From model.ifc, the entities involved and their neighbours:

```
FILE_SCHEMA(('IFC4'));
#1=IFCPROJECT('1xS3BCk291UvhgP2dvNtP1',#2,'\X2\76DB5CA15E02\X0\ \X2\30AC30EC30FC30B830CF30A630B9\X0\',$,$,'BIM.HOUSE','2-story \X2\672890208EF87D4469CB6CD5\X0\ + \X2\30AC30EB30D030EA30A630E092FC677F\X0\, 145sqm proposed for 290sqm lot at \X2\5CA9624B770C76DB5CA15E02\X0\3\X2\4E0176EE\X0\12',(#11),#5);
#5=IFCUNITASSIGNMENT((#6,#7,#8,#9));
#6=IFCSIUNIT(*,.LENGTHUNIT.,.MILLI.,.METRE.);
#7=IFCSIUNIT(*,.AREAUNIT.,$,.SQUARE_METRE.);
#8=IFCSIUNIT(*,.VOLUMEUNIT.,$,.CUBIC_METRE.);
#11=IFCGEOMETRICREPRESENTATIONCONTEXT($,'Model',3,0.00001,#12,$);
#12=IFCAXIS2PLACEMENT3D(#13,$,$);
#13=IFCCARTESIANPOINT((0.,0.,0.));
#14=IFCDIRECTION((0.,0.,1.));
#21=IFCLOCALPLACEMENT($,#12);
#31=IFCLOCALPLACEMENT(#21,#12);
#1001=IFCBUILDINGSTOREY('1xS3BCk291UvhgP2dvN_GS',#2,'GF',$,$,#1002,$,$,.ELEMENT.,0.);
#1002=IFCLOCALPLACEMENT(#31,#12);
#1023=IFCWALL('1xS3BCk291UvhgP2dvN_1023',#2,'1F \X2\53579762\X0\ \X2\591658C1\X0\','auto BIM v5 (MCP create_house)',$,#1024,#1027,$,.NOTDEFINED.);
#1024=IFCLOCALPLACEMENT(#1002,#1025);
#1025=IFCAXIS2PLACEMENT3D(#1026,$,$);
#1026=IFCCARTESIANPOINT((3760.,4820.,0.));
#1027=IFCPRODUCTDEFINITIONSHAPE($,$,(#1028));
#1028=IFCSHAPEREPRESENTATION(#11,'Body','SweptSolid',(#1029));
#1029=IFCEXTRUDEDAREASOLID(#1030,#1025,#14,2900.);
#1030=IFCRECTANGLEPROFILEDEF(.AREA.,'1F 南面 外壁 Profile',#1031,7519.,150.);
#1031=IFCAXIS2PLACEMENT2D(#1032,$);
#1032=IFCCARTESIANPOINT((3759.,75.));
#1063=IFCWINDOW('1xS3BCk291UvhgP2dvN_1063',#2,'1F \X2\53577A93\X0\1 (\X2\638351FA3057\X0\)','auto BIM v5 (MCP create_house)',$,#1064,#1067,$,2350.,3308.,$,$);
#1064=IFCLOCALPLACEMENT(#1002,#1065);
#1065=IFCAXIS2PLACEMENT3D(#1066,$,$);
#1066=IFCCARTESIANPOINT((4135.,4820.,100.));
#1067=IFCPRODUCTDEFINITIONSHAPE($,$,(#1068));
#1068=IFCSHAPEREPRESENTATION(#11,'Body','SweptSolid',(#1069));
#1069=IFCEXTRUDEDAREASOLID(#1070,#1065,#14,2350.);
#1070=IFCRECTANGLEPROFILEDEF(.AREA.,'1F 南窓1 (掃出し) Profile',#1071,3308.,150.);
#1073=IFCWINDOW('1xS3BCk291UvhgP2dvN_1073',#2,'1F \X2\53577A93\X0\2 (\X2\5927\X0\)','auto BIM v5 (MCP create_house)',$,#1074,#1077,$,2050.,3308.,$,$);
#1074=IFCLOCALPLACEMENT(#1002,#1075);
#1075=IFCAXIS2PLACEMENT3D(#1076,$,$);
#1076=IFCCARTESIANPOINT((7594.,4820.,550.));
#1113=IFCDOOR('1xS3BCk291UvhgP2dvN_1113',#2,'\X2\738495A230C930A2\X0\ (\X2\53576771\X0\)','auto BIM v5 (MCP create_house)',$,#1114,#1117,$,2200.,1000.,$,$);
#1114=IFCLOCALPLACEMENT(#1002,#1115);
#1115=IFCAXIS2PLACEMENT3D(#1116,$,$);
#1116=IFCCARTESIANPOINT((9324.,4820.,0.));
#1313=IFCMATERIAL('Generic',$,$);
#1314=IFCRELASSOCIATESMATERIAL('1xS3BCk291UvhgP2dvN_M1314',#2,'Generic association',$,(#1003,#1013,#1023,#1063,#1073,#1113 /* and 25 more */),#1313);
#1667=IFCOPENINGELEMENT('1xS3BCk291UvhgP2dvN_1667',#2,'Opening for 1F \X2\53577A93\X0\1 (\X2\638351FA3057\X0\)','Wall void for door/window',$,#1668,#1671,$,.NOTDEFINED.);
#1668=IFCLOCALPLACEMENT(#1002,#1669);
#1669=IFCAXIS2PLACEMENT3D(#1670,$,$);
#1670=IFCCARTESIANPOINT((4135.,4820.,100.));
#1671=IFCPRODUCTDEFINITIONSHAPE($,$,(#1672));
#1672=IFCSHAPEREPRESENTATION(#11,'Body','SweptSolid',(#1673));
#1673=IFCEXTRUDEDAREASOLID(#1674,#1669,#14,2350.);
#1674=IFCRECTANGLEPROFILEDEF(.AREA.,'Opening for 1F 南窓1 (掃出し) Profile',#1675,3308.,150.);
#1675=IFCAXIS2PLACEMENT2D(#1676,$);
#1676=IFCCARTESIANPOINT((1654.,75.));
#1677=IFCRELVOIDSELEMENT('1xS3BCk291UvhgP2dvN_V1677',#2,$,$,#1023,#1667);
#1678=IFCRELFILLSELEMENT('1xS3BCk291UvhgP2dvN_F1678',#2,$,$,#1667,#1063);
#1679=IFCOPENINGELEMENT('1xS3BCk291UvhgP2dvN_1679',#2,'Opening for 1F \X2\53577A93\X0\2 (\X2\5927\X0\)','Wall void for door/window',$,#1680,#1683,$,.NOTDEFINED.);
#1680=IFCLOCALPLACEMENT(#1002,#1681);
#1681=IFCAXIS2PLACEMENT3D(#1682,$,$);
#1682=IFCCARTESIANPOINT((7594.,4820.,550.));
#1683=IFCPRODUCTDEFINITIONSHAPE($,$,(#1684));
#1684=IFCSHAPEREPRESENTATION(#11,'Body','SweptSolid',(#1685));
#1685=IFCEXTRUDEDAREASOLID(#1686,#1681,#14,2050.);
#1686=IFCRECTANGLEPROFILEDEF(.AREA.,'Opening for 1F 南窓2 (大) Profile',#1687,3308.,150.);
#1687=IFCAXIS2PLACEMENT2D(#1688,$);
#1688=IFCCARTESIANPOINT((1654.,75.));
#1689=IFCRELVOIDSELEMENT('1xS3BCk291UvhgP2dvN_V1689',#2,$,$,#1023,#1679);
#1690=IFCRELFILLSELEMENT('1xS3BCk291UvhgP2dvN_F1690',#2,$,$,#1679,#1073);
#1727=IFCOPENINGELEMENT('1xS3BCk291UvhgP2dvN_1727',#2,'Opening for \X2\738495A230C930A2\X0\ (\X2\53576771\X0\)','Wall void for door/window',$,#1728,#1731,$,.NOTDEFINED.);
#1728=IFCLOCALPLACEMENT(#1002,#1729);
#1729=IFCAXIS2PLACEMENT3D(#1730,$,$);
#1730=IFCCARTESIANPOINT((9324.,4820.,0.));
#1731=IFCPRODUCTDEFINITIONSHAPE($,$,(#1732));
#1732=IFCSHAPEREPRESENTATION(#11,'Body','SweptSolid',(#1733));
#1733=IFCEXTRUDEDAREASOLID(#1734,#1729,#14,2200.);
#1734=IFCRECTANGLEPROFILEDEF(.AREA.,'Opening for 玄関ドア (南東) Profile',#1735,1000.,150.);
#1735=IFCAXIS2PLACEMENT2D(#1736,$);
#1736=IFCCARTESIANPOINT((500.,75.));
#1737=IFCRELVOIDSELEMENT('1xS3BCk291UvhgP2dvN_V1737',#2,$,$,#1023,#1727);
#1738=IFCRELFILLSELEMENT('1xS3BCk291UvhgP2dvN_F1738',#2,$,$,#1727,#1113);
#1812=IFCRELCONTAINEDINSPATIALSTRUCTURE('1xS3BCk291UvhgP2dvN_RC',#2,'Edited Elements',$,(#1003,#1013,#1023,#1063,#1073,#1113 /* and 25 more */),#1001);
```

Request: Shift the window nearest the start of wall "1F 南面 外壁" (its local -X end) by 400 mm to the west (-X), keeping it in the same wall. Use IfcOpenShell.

```python
import ifcopenshell
import ifcopenshell.api.geometry
import ifcopenshell.util.placement

model = ifcopenshell.open("model.ifc")

window = model.by_id(1063)
opening = window.FillsVoids[0].RelatingOpeningElement
wall = opening.VoidsElements[0].RelatingBuildingElement

wall_matrix = ifcopenshell.util.placement.get_local_placement(wall.ObjectPlacement)
shift = wall_matrix[:3, 0] * -400.0
before = ifcopenshell.util.placement.get_local_placement(window.ObjectPlacement)[:3, 3].copy()

# The window is not placed relative to its opening, so move both.
for product in (opening, window):
    matrix = ifcopenshell.util.placement.get_local_placement(product.ObjectPlacement)
    matrix[:3, 3] += shift
    ifcopenshell.api.geometry.edit_object_placement(model, product=product, matrix=matrix, is_si=False)

after = ifcopenshell.util.placement.get_local_placement(window.ObjectPlacement)[:3, 3]
print("window moved by", (after - before).round(3) + 0.0)

model.write("model_rev.ifc")
```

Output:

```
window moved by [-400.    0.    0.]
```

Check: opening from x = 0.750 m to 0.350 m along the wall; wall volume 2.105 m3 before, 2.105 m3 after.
